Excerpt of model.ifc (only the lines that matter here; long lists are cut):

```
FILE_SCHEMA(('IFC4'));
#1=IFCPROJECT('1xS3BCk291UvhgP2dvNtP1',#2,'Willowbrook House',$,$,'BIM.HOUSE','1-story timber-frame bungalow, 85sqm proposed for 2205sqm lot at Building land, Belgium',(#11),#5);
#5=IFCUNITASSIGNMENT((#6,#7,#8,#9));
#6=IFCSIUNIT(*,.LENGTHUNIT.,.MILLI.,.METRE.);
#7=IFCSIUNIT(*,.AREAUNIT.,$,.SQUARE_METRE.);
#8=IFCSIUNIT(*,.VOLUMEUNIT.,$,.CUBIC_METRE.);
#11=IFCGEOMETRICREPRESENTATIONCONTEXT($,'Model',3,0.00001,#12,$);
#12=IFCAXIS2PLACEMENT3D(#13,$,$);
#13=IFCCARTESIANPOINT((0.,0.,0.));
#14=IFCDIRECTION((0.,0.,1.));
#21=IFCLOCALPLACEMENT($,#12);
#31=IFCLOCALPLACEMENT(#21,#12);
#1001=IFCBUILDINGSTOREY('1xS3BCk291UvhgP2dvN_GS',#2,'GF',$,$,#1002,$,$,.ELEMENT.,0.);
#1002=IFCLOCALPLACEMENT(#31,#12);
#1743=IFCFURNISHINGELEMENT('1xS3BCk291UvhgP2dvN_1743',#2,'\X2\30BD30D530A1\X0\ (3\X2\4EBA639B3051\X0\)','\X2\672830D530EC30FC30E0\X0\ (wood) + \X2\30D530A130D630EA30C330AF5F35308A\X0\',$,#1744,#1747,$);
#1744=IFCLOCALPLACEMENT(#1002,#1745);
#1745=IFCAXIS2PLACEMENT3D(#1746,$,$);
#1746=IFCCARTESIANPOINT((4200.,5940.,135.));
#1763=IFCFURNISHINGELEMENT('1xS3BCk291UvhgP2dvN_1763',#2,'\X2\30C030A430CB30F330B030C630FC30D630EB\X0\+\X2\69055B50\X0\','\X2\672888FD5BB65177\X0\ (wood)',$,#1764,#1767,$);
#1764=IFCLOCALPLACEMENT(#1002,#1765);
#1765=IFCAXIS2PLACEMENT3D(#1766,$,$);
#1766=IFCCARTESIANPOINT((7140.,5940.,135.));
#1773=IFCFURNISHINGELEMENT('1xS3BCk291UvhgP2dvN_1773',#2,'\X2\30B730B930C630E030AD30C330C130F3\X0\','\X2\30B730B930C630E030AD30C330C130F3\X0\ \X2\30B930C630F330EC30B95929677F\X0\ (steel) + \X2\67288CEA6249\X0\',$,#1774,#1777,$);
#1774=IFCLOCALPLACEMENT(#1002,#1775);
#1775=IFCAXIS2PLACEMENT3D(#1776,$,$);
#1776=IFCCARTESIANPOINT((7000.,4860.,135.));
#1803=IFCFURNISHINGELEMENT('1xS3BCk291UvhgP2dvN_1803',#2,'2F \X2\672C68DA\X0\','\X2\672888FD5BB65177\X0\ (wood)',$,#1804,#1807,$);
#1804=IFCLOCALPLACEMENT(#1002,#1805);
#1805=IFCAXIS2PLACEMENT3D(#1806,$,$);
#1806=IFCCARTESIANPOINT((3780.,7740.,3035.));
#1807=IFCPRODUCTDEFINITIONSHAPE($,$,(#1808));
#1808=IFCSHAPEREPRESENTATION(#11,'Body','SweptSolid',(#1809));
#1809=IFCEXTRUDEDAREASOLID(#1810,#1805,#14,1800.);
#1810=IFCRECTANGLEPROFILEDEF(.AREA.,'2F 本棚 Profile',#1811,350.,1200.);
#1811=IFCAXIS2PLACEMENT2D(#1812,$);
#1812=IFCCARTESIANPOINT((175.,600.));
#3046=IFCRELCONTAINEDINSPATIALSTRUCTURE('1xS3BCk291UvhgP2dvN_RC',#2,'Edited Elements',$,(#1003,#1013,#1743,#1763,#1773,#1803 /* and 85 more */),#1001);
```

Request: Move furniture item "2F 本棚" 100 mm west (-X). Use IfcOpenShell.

```python
import ifcopenshell
import ifcopenshell.api.geometry
import ifcopenshell.util.placement
import ifcopenshell.util.unit

model = ifcopenshell.open("model.ifc")
unit_scale = ifcopenshell.util.unit.calculate_unit_scale(model)

item = model.by_guid("1xS3BCk291UvhgP2dvN_1803")
matrix = ifcopenshell.util.placement.get_local_placement(item.ObjectPlacement)
matrix[0, 3] -= 0.1 / unit_scale
ifcopenshell.api.geometry.edit_object_placement(model, product=item, matrix=matrix, is_si=False)

print(ifcopenshell.util.placement.get_local_placement(item.ObjectPlacement).round(3) + 0.0)

model.write("model_rev.ifc")
```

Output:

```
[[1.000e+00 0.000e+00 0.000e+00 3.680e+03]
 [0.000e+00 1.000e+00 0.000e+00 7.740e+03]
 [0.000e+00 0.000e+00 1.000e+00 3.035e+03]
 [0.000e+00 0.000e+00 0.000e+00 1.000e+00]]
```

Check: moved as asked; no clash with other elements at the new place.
